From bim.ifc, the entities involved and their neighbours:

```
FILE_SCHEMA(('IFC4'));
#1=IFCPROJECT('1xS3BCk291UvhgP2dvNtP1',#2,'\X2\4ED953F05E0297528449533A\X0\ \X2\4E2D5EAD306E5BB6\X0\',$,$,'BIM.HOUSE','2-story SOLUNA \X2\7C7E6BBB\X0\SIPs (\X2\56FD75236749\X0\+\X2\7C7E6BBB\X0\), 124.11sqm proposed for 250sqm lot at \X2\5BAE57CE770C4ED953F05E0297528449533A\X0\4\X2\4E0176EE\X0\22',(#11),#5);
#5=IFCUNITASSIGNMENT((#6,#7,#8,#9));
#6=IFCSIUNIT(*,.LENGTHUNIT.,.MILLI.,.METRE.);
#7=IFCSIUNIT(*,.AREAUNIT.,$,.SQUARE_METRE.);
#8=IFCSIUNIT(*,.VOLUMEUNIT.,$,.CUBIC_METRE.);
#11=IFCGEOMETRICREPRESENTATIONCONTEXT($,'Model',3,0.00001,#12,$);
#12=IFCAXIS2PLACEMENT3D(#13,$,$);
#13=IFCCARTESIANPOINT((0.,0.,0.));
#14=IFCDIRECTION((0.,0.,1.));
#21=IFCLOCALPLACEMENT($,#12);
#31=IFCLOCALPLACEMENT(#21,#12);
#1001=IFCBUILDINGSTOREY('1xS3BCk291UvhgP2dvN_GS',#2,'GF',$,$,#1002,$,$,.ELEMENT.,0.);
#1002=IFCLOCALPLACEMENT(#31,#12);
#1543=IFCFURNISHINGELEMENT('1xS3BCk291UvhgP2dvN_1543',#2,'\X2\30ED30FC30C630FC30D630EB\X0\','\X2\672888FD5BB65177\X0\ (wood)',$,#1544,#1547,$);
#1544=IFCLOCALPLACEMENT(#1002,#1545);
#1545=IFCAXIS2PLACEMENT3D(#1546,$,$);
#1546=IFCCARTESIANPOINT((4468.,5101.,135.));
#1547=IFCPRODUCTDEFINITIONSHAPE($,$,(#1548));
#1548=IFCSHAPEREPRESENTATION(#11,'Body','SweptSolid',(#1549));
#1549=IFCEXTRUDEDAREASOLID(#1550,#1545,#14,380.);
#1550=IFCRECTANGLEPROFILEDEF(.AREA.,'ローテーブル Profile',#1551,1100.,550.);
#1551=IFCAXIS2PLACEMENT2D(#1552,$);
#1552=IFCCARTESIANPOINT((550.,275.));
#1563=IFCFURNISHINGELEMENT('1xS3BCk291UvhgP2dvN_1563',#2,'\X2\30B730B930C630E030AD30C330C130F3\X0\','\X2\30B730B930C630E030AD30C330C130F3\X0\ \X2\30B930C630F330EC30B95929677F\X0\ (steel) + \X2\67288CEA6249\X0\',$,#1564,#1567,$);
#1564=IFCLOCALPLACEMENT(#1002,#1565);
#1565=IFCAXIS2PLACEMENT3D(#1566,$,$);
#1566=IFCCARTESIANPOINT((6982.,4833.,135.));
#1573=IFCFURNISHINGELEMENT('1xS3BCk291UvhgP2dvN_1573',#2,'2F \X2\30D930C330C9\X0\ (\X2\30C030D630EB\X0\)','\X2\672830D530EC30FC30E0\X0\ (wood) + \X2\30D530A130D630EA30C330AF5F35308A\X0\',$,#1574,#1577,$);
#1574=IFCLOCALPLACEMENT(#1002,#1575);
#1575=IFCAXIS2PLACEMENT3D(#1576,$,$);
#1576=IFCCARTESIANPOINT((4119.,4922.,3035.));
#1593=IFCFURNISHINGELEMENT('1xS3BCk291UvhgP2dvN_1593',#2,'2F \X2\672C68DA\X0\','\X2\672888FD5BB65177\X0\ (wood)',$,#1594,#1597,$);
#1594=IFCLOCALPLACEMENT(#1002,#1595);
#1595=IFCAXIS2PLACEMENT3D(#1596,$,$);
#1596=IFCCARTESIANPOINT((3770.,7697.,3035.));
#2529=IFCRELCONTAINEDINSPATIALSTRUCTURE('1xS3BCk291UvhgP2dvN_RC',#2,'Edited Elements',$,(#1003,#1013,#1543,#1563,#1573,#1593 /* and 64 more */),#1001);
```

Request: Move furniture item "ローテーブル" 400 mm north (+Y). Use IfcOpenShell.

```python
import ifcopenshell
import ifcopenshell.api.geometry
import ifcopenshell.util.placement
import ifcopenshell.util.unit

model = ifcopenshell.open("bim.ifc")
unit_scale = ifcopenshell.util.unit.calculate_unit_scale(model)

item = model.by_guid("1xS3BCk291UvhgP2dvN_1543")
matrix = ifcopenshell.util.placement.get_local_placement(item.ObjectPlacement)
matrix[1, 3] += 0.4 / unit_scale
ifcopenshell.api.geometry.edit_object_placement(model, product=item, matrix=matrix, is_si=False)

print(ifcopenshell.util.placement.get_local_placement(item.ObjectPlacement).round(3) + 0.0)

model.write("bim_rev.ifc")
```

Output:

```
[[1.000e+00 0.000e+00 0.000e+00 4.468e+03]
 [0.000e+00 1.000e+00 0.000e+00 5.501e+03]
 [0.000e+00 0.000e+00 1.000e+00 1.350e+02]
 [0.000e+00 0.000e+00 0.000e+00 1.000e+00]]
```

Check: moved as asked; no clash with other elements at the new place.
